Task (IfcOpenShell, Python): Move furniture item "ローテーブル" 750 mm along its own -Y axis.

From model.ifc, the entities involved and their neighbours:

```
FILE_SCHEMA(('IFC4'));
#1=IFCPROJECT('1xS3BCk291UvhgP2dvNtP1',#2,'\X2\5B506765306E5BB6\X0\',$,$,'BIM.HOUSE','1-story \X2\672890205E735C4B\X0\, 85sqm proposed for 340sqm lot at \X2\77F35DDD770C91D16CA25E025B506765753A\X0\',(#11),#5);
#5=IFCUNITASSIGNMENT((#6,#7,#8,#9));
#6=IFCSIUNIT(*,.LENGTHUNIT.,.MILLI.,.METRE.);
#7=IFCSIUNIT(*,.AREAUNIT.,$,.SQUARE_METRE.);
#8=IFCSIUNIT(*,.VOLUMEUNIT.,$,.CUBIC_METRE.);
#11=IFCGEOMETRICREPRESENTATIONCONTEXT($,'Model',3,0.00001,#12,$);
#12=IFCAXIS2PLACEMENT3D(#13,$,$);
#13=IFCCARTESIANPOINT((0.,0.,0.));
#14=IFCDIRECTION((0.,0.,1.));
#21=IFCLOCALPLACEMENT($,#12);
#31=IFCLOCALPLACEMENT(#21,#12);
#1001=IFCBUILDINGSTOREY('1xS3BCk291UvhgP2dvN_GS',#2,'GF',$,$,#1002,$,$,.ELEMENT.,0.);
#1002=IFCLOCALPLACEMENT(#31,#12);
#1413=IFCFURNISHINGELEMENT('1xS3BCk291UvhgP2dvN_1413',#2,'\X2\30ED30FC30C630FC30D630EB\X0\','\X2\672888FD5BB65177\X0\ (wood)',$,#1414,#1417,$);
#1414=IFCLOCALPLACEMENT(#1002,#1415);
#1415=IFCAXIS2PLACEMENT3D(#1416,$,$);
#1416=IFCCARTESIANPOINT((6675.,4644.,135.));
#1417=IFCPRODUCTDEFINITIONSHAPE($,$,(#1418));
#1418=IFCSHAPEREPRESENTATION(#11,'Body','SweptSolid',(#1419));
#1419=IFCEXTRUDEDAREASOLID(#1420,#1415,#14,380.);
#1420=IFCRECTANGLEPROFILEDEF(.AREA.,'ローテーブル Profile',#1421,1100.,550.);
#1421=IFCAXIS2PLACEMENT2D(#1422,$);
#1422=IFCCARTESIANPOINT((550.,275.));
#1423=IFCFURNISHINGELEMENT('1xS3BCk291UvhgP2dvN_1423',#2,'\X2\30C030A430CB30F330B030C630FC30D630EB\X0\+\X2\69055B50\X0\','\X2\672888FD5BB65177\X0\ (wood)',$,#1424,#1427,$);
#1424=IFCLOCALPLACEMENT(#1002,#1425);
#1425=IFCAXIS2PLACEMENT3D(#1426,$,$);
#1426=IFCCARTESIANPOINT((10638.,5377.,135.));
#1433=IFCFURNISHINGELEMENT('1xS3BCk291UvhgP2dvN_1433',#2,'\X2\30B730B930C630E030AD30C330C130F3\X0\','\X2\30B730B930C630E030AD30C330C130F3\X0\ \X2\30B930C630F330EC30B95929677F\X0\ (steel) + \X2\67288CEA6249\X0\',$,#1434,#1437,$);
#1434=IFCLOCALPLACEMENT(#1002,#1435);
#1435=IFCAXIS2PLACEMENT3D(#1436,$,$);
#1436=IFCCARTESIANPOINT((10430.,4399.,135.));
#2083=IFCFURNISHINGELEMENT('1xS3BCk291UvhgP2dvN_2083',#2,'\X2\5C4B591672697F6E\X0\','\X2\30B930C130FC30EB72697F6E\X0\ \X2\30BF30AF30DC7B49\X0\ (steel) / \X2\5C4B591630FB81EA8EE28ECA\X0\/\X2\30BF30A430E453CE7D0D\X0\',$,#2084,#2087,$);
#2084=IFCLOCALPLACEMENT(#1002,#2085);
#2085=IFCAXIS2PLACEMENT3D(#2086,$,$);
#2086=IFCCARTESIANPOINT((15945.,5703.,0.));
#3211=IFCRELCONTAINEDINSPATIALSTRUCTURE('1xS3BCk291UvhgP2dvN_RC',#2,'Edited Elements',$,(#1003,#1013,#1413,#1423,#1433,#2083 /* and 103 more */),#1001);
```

```python
import ifcopenshell
import ifcopenshell.api.geometry
import ifcopenshell.util.placement

model = ifcopenshell.open("model.ifc")

item = model.by_id(1413)
matrix = ifcopenshell.util.placement.get_local_placement(item.ObjectPlacement)
matrix[:3, 3] -= matrix[:3, 1] * 750.0
ifcopenshell.api.geometry.edit_object_placement(model, product=item, matrix=matrix, is_si=False)

print(ifcopenshell.util.placement.get_local_placement(item.ObjectPlacement).round(3) + 0.0)

model.write("model_rev.ifc")
```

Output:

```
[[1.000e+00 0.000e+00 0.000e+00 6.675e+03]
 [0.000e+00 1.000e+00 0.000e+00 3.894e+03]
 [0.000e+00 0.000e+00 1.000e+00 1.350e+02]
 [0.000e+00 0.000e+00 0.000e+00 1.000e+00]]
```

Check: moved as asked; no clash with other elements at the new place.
